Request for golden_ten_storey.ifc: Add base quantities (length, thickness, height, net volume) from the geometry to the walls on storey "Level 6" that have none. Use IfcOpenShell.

First a look at what the model holds.

```python
import ifcopenshell
import ifcopenshell.util.element
import ifcopenshell.util.unit

model = ifcopenshell.open("golden_ten_storey.ifc")
print(model.schema)
for unit_type in ("LENGTHUNIT", "AREAUNIT", "VOLUMEUNIT"):
    print(unit_type, ifcopenshell.util.unit.calculate_unit_scale(model, unit_type))
storey = next(s for s in model.by_type("IfcBuildingStorey") if s.Name == "Level 6")
walls = [e for e in ifcopenshell.util.element.get_decomposition(storey) if e.is_a("IfcWall")]
for e in sorted(walls, key=lambda e: e.id()):
    print(e.id(), e.is_a(), e.Name, list(ifcopenshell.util.element.get_psets(e, qtos_only=True)), sep=" | ")
```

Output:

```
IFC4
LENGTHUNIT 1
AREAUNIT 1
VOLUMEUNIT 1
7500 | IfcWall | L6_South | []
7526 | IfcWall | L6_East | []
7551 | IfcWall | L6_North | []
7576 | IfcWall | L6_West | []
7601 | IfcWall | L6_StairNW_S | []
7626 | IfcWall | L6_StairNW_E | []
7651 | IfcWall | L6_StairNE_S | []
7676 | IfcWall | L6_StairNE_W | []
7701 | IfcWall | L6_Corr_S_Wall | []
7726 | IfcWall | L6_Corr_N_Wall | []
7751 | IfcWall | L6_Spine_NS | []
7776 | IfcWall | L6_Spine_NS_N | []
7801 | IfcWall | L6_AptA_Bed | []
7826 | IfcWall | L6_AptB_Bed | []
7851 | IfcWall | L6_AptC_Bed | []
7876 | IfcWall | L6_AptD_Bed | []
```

```python
import ifcopenshell
import ifcopenshell.api.pset
import ifcopenshell.geom
import ifcopenshell.util.element
import ifcopenshell.util.shape
import ifcopenshell.util.unit

model = ifcopenshell.open("golden_ten_storey.ifc")
unit_scale = ifcopenshell.util.unit.calculate_unit_scale(model)
volume_scale = ifcopenshell.util.unit.calculate_unit_scale(model, "VOLUMEUNIT")
settings = ifcopenshell.geom.settings()

storey = next(s for s in model.by_type("IfcBuildingStorey") if s.Name == "Level 6")
walls = [e for e in ifcopenshell.util.element.get_decomposition(storey) if e.is_a("IfcWall")]

for e in sorted(walls, key=lambda e: e.id()):
    if ifcopenshell.util.element.get_psets(e, qtos_only=True, should_inherit=False):
        continue
    # Geometry comes back in metres, in the element's own axes.
    shape = ifcopenshell.geom.create_shape(settings, e)
    values = {
        "Length": ifcopenshell.util.shape.get_x(shape.geometry) / unit_scale,
        "Width": ifcopenshell.util.shape.get_y(shape.geometry) / unit_scale,
        "Height": ifcopenshell.util.shape.get_z(shape.geometry) / unit_scale,
        "NetVolume": ifcopenshell.util.shape.get_volume(shape.geometry) / volume_scale,
    }
    qto = ifcopenshell.api.pset.add_qto(model, product=e, name="Qto_WallBaseQuantities")
    ifcopenshell.api.pset.edit_qto(model, qto=qto, properties=values)
    print(e.id(), {k: round(v, 3) for k, v in values.items()})

model.write("golden_ten_storey-out.ifc")
```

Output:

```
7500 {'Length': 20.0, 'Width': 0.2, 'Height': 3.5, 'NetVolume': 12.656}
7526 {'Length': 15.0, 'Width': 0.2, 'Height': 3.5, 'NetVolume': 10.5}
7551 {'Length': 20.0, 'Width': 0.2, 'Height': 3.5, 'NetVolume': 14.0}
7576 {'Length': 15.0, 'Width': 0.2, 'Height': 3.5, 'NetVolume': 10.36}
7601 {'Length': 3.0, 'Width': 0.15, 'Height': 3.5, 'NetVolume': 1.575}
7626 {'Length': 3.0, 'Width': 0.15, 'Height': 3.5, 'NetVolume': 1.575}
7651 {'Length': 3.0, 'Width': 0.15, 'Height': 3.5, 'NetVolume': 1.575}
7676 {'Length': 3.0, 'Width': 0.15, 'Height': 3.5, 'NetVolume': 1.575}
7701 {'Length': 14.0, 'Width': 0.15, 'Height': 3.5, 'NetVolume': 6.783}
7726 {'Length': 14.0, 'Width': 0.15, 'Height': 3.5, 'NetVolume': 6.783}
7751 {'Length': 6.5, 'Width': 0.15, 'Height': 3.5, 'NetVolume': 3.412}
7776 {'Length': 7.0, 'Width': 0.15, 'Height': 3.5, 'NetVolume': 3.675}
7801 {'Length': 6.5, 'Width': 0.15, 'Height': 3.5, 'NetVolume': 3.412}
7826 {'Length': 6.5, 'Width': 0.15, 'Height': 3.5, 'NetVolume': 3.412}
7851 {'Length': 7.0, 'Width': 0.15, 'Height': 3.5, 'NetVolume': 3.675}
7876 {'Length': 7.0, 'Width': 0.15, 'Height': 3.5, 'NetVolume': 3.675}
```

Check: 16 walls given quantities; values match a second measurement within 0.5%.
